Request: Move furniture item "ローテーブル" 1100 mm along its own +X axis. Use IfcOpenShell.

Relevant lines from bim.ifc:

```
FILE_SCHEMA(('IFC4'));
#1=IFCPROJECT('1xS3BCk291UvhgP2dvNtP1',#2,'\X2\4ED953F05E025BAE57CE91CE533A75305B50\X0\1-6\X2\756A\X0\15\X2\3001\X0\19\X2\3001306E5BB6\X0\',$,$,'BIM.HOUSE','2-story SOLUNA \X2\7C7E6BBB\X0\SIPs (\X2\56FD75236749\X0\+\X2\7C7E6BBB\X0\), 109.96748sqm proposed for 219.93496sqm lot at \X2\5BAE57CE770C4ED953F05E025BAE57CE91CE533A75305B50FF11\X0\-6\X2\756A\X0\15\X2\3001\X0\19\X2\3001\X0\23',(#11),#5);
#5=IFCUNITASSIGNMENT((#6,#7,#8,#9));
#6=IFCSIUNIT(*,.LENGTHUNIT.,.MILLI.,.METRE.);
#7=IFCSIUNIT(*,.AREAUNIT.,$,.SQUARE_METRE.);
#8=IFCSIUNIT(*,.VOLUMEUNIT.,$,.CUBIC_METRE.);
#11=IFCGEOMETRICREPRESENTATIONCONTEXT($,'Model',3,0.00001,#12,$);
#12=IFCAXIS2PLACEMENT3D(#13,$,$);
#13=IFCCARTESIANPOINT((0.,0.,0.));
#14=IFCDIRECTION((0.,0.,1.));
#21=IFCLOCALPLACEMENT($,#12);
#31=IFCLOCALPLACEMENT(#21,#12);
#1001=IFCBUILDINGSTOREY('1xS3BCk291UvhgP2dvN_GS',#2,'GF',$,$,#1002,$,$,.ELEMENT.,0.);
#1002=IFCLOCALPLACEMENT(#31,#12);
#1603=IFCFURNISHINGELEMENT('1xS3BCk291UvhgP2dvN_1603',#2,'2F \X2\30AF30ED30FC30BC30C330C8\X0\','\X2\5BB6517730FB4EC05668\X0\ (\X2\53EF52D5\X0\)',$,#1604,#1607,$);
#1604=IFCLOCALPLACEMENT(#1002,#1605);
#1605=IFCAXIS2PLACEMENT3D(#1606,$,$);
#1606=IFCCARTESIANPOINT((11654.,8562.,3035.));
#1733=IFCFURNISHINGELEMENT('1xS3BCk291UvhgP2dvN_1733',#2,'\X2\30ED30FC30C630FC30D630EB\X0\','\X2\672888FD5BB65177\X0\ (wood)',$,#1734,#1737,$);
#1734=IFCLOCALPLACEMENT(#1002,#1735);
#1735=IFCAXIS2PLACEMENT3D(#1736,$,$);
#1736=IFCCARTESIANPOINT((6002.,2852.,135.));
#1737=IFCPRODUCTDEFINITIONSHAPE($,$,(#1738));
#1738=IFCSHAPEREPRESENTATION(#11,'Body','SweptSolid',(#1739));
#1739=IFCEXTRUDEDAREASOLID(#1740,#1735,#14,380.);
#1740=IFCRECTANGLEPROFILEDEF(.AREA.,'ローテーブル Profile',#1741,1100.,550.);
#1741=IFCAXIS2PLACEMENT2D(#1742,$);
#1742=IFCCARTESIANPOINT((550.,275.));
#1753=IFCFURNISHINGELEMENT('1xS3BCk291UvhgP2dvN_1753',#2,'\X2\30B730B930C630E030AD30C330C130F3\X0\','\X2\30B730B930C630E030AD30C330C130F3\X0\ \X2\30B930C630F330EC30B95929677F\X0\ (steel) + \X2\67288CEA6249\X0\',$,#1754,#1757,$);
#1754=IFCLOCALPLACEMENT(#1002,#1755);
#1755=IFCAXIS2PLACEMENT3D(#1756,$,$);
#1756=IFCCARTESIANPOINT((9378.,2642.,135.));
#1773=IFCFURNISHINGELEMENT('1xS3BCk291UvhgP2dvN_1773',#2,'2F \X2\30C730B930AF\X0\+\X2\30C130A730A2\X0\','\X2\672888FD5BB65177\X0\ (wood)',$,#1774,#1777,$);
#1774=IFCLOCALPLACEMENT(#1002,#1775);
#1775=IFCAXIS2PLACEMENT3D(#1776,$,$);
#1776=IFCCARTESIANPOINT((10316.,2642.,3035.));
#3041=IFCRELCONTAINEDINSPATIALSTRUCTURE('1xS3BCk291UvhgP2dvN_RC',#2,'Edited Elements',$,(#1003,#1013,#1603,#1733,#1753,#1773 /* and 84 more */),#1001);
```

```python
import ifcopenshell
import ifcopenshell.api.geometry
import ifcopenshell.util.placement
import ifcopenshell.util.unit

model = ifcopenshell.open("bim.ifc")
unit_scale = ifcopenshell.util.unit.calculate_unit_scale(model)

item = model.by_guid("1xS3BCk291UvhgP2dvN_1733")
matrix = ifcopenshell.util.placement.get_local_placement(item.ObjectPlacement)
matrix[:3, 3] += matrix[:3, 0] * 1.1 / unit_scale
ifcopenshell.api.geometry.edit_object_placement(model, product=item, matrix=matrix, is_si=False)

print(ifcopenshell.util.placement.get_local_placement(item.ObjectPlacement).round(3) + 0.0)

model.write("bim-out.ifc")
```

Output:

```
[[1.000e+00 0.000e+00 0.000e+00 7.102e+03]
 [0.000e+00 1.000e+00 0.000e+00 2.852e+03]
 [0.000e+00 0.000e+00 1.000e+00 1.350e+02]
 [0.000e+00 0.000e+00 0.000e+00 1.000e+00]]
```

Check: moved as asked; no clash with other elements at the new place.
